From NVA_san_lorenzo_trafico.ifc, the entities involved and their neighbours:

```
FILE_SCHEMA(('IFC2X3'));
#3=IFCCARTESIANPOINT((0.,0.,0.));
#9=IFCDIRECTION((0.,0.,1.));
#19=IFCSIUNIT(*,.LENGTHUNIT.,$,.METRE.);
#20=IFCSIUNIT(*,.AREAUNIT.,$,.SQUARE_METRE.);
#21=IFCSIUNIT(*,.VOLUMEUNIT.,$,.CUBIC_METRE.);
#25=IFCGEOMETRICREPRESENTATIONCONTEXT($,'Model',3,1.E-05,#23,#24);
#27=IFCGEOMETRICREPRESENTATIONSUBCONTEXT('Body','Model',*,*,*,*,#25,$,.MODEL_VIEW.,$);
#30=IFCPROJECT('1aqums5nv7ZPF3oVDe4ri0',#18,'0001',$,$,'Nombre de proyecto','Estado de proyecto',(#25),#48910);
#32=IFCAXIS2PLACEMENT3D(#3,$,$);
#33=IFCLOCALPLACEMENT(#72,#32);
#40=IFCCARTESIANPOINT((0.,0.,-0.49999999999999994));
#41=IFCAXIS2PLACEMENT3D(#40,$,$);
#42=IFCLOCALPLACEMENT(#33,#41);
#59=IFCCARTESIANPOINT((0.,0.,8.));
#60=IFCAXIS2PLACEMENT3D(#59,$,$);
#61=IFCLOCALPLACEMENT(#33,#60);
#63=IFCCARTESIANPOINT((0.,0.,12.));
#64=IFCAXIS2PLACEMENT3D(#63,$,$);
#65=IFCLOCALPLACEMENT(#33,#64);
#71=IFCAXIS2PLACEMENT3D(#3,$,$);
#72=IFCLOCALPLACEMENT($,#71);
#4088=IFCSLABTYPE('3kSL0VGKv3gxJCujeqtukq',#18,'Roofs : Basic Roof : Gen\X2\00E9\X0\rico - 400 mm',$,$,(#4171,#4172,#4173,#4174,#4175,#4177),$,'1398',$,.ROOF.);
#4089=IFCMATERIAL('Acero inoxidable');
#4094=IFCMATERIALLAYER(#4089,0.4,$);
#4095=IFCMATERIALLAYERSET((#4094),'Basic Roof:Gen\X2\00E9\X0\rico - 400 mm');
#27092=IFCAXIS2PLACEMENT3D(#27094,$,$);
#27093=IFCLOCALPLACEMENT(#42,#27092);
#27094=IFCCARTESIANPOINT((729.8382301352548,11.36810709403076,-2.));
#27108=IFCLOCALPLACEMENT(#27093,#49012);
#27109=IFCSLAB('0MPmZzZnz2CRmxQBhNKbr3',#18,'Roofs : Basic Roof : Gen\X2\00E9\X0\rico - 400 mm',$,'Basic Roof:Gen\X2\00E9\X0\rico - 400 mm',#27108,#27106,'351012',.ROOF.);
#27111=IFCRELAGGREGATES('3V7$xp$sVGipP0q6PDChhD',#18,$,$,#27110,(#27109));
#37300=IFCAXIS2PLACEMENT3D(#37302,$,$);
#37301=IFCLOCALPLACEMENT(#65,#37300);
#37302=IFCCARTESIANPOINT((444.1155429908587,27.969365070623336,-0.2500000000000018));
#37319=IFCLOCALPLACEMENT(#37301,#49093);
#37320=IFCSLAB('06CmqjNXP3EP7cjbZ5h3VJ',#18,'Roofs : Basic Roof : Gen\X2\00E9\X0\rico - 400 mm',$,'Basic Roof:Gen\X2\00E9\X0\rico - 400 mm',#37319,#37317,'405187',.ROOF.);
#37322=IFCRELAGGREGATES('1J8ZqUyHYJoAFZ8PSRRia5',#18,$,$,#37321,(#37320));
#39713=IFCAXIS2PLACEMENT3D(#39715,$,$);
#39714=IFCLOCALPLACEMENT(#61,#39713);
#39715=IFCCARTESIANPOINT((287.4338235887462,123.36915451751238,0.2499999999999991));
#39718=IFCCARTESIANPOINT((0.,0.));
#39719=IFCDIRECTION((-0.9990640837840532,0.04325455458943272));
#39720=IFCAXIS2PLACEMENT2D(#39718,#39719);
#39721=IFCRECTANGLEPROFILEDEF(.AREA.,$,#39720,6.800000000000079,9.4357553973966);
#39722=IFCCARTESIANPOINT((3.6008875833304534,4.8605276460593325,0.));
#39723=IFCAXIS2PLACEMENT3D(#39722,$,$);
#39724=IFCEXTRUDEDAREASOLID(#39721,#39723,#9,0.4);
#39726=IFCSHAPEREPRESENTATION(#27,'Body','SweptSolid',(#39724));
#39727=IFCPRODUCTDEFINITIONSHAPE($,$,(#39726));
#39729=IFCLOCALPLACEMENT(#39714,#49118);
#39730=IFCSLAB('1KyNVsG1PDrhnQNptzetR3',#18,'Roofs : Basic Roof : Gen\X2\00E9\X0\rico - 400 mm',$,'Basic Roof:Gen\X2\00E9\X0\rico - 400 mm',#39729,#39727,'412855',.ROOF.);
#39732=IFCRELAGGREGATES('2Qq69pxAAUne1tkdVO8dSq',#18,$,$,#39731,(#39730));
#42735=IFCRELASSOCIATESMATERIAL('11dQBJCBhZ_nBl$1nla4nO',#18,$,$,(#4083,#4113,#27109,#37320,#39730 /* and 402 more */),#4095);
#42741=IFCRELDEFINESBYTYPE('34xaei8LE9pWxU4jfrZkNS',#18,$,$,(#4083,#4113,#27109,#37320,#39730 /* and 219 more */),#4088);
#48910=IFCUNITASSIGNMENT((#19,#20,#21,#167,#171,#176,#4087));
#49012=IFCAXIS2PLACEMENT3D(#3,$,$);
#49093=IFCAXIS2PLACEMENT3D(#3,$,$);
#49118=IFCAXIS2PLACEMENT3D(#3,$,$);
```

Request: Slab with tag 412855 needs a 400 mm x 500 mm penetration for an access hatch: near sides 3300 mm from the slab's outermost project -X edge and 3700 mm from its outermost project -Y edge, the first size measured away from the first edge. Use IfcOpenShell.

```python
import numpy as np
import ifcopenshell
import ifcopenshell.api.feature
import ifcopenshell.api.geometry
import ifcopenshell.api.root
import ifcopenshell.geom
import ifcopenshell.util.placement
import ifcopenshell.util.representation
import ifcopenshell.util.shape
import ifcopenshell.util.unit

model = ifcopenshell.open("NVA_san_lorenzo_trafico.ifc")
unit_scale = ifcopenshell.util.unit.calculate_unit_scale(model)
settings = ifcopenshell.geom.settings()


def volume(element):
    """Net volume in cubic metres, openings subtracted."""
    shape = ifcopenshell.geom.create_shape(settings, element)
    return ifcopenshell.util.shape.get_volume(shape.geometry)


slab = model.by_id(39730)
before = volume(slab)

# Extent in the slab's own axes, in metres. The edges named are its -X and -Y sides.
slab_shape = ifcopenshell.geom.create_shape(settings, slab)
vertices = ifcopenshell.util.shape.get_vertices(slab_shape.geometry)
x_min, y_min, bottom = vertices.min(axis=0)
top = vertices[:, 2].max()

opening = ifcopenshell.api.root.create_entity(model, ifc_class="IfcOpeningElement", name="Access hatch opening")
context = ifcopenshell.util.representation.get_context(model, "Model", "Body", "MODEL_VIEW")
width, depth = 0.4, 0.5
outline = [(0.0, 0.0), (width, 0.0), (width, depth), (0.0, depth), (0.0, 0.0)]
# Overshoot both faces by 50 mm so the cut is clean.
shape = ifcopenshell.api.geometry.add_slab_representation(
    model, context=context, depth=top - bottom + 0.1, polyline=outline
)
ifcopenshell.api.geometry.assign_representation(model, product=opening, representation=shape)

matrix = ifcopenshell.util.placement.get_local_placement(slab.ObjectPlacement)
matrix[:, 3] = matrix @ np.append(np.array([x_min + 3.3, y_min + 3.7, bottom - 0.05]) / unit_scale, 1.0)
ifcopenshell.api.geometry.edit_object_placement(model, product=opening, matrix=matrix, is_si=False)
ifcopenshell.api.feature.add_feature(model, feature=opening, element=slab)

after = volume(slab)

print(f"slab volume {before:.3f} -> {after:.3f} m3")

model.write("NVA_san_lorenzo_trafico_v2.ifc")
```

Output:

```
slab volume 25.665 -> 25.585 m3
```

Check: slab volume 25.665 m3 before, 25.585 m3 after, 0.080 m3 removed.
